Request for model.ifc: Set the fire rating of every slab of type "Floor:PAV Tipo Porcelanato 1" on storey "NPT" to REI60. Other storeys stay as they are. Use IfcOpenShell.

First a look at what the model holds.

```python
import ifcopenshell
import ifcopenshell.util.element

model = ifcopenshell.open("model.ifc")
print(model.schema)
storey = next(s for s in model.by_type("IfcBuildingStorey") if s.Name == "NPT")
slabs = [e for e in ifcopenshell.util.element.get_decomposition(storey) if e.is_a("IfcSlab")]
seen = {}
for e in slabs:
    element_type = ifcopenshell.util.element.get_type(e)
    key = (element_type.Name if element_type != e and element_type else None, ifcopenshell.util.element.get_pset(e, "Pset_SlabCommon", "FireRating"))
    seen[key] = seen.get(key, 0) + 1
for (name, value), count in sorted(seen.items(), key=str):
    print(count, "x", name, "|", value)
```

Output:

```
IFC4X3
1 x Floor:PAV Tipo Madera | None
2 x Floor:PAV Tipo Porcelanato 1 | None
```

```python
import ifcopenshell
import ifcopenshell.api.pset
import ifcopenshell.util.element

model = ifcopenshell.open("model.ifc")

storey = next(s for s in model.by_type("IfcBuildingStorey") if s.Name == "NPT")
slabs = [e for e in ifcopenshell.util.element.get_decomposition(storey) if e.is_a("IfcSlab")]

count = 0
for e in slabs:
    element_type = ifcopenshell.util.element.get_type(e)
    if element_type in (None, e) or element_type.Name != "Floor:PAV Tipo Porcelanato 1":
        continue
    # add_pset returns the element's existing set when there is one.
    pset = ifcopenshell.api.pset.add_pset(model, product=e, name="Pset_SlabCommon")
    ifcopenshell.api.pset.edit_pset(model, pset=pset, properties={"FireRating": "REI60"})
    count += 1

print(count, "slabs updated")

model.write("model_edited.ifc")
```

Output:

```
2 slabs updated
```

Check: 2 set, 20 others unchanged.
